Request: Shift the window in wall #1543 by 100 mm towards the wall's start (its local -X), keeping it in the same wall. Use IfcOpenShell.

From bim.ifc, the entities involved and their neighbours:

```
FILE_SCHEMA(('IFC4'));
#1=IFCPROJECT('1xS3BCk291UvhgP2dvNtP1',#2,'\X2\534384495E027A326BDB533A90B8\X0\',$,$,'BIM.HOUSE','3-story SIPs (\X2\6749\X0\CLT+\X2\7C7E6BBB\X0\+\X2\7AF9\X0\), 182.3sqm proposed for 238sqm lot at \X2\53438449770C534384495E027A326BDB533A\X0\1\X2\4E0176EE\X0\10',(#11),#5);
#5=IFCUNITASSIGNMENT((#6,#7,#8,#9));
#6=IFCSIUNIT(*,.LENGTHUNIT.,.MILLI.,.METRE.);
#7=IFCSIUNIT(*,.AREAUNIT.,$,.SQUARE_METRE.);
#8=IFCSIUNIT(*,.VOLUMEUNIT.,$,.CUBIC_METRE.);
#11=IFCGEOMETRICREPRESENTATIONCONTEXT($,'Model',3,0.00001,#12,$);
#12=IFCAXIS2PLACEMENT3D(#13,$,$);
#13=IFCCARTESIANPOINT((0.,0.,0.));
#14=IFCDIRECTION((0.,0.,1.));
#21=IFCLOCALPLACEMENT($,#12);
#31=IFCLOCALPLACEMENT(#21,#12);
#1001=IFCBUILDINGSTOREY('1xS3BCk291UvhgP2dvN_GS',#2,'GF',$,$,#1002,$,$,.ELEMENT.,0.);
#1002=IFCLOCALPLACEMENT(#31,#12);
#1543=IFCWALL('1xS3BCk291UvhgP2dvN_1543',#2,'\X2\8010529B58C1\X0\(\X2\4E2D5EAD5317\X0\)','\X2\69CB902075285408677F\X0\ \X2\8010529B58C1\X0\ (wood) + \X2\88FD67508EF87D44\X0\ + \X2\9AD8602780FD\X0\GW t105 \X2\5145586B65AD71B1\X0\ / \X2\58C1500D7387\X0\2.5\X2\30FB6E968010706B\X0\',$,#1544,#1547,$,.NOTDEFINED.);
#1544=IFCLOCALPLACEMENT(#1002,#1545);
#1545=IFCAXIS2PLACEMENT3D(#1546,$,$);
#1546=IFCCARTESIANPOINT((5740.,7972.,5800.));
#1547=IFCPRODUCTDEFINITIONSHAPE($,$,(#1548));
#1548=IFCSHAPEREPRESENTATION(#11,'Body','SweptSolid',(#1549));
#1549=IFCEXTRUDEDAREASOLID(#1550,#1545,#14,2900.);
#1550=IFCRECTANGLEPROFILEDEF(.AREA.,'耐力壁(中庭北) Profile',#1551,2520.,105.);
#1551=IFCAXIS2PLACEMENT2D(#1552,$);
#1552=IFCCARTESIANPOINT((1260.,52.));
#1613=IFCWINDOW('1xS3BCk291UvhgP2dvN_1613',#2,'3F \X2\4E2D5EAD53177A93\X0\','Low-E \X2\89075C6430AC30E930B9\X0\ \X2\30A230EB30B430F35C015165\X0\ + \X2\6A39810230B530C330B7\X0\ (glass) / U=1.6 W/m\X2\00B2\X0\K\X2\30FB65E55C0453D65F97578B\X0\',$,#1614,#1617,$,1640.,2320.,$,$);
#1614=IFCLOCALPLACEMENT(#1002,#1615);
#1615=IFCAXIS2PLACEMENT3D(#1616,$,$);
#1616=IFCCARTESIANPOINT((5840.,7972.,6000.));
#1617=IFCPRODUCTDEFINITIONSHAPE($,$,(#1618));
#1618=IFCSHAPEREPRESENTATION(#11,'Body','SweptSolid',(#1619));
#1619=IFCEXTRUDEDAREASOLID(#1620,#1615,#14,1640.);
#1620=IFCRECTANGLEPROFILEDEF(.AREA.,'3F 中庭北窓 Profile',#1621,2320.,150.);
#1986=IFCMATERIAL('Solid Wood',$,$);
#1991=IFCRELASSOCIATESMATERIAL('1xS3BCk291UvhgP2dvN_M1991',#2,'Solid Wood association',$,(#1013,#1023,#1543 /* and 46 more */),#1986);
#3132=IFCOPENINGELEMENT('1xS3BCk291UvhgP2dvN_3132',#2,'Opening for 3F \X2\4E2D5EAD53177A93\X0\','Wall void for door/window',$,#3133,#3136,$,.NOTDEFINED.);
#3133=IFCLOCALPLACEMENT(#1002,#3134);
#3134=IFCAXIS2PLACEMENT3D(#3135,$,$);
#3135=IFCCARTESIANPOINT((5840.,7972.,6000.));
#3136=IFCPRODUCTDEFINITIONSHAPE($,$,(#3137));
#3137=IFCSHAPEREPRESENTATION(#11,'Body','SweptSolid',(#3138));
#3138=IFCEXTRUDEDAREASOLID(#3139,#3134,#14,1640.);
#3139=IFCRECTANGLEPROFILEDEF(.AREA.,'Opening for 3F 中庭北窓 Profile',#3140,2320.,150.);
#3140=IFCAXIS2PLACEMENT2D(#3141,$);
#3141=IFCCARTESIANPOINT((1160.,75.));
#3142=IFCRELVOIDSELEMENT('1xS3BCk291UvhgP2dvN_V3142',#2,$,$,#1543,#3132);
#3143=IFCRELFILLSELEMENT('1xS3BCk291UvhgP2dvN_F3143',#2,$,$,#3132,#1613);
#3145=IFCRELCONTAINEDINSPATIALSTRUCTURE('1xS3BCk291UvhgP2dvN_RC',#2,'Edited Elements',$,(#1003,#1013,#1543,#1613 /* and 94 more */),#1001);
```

```python
import ifcopenshell
import ifcopenshell.api.geometry
import ifcopenshell.util.placement
import ifcopenshell.util.unit

model = ifcopenshell.open("bim.ifc")
unit_scale = ifcopenshell.util.unit.calculate_unit_scale(model)

window = model.by_guid("1xS3BCk291UvhgP2dvN_1613")
opening = window.FillsVoids[0].RelatingOpeningElement
wall = opening.VoidsElements[0].RelatingBuildingElement

wall_matrix = ifcopenshell.util.placement.get_local_placement(wall.ObjectPlacement)
shift = wall_matrix[:3, 0] * -0.1 / unit_scale
before = ifcopenshell.util.placement.get_local_placement(window.ObjectPlacement)[:3, 3].copy()

# The window is not placed relative to its opening, so move both.
for product in (opening, window):
    matrix = ifcopenshell.util.placement.get_local_placement(product.ObjectPlacement)
    matrix[:3, 3] += shift
    ifcopenshell.api.geometry.edit_object_placement(model, product=product, matrix=matrix, is_si=False)

after = ifcopenshell.util.placement.get_local_placement(window.ObjectPlacement)[:3, 3]
print("window moved by", (after - before).round(3) + 0.0)

model.write("bim_edited.ifc")
```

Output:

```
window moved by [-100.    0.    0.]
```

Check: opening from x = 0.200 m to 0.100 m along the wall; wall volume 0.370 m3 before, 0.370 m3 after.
